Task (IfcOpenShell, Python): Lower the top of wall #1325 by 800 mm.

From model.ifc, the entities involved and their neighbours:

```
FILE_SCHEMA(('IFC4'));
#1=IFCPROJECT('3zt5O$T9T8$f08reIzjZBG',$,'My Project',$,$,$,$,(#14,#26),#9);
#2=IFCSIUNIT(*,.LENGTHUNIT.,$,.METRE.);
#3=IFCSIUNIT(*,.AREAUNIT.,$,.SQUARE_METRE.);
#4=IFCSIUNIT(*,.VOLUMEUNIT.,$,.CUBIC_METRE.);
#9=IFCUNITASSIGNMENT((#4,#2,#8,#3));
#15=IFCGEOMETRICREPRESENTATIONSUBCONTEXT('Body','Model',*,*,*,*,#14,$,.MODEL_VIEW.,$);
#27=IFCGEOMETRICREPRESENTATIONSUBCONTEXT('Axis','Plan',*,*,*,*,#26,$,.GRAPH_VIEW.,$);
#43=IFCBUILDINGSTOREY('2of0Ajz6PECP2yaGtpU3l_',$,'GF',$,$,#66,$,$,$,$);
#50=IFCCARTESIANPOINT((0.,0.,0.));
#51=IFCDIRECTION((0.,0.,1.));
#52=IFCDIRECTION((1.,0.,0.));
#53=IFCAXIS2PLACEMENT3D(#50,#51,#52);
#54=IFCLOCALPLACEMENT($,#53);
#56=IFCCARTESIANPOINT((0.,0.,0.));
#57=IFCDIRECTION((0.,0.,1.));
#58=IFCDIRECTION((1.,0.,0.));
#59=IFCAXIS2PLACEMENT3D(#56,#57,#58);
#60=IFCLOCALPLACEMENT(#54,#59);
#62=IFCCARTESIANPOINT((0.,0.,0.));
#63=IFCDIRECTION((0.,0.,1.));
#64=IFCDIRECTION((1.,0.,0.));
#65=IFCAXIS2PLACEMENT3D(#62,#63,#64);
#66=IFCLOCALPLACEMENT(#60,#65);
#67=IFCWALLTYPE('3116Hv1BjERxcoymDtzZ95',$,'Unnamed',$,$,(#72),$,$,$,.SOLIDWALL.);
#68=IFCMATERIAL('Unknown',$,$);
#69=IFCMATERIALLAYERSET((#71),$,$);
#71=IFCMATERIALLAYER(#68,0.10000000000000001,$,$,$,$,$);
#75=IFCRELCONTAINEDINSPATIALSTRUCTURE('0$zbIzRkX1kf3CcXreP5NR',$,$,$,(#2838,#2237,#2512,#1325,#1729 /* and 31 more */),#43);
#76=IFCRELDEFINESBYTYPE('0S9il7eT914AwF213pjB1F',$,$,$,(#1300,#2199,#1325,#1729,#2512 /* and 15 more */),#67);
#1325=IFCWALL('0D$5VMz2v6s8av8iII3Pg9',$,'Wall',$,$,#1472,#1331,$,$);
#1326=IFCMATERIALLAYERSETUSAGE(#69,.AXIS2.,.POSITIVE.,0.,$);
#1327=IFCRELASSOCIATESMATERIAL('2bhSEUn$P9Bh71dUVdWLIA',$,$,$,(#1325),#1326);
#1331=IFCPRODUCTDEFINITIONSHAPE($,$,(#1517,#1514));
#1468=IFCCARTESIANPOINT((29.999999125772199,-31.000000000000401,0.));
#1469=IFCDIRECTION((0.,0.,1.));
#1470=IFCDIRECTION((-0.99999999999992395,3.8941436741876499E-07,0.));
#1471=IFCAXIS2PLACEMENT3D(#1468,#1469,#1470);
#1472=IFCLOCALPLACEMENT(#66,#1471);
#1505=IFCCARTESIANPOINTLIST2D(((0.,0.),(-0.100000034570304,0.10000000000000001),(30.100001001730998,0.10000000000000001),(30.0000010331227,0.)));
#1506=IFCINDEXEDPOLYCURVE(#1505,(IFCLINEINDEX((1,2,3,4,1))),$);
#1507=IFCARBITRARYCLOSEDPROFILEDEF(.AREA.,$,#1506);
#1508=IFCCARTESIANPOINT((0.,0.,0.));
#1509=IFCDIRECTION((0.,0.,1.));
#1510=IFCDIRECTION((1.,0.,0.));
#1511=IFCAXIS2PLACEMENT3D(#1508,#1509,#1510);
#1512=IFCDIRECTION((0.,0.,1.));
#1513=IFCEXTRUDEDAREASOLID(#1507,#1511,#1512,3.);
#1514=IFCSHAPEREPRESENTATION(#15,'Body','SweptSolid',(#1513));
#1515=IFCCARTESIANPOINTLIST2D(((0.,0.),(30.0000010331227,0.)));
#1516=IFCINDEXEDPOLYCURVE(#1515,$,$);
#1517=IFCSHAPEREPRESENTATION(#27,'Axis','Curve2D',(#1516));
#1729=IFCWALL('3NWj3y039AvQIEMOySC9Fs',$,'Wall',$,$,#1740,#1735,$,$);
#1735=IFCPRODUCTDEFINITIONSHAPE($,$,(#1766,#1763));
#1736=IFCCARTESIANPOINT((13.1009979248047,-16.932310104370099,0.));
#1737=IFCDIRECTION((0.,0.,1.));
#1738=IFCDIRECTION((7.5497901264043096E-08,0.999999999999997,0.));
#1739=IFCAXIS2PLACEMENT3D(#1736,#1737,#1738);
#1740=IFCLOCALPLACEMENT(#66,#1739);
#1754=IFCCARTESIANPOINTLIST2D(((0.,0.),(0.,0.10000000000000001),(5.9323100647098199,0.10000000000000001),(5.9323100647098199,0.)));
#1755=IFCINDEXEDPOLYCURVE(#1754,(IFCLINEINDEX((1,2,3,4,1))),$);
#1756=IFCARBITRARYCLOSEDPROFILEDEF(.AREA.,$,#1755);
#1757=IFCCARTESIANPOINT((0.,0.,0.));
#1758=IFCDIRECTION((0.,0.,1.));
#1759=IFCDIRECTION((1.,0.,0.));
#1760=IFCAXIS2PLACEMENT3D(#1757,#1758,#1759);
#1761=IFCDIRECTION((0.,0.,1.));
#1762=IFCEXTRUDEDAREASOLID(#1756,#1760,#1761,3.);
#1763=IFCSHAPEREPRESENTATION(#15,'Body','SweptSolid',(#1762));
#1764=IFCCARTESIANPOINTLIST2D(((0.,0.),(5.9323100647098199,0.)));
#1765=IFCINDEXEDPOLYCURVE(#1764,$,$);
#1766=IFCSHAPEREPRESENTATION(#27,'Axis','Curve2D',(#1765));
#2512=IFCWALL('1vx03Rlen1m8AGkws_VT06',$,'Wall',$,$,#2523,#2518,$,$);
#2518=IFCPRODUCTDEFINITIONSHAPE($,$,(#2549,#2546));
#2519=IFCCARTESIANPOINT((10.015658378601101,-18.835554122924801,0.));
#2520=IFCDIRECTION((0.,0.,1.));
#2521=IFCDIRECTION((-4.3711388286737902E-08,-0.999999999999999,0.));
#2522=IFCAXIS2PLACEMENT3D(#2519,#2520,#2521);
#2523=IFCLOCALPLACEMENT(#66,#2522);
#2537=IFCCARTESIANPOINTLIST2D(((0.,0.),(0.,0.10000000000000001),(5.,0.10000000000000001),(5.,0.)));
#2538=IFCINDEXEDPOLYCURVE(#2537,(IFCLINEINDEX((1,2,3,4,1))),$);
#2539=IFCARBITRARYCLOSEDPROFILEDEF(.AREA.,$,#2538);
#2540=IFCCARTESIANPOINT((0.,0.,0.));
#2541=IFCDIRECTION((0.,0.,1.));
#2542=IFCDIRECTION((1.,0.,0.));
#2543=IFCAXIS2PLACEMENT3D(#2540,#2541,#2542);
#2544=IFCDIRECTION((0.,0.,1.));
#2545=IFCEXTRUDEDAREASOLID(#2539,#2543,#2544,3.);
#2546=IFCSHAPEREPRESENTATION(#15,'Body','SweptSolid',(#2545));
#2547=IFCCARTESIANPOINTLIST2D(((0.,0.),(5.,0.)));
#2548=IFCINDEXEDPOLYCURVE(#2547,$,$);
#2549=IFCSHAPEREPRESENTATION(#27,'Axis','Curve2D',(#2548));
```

```python
import ifcopenshell
import ifcopenshell.geom
import ifcopenshell.util.representation
import ifcopenshell.util.shape
import ifcopenshell.util.unit

model = ifcopenshell.open("model.ifc")
unit_scale = ifcopenshell.util.unit.calculate_unit_scale(model)
settings = ifcopenshell.geom.settings()


def volume(element):
    """Net volume in cubic metres, openings subtracted."""
    shape = ifcopenshell.geom.create_shape(settings, element)
    return ifcopenshell.util.shape.get_volume(shape.geometry)


wall = model.by_guid("0D$5VMz2v6s8av8iII3Pg9")
before = volume(wall)

body = ifcopenshell.util.representation.get_representation(wall, "Model", "Body")
solid = body.Items[0]
old_height = solid.Depth
solid.Depth -= 0.8 / unit_scale
after = volume(wall)

print(f"height {old_height:g} -> {solid.Depth:g}, volume {before:.3f} -> {after:.3f} m3")

model.write("model_v2.ifc")
```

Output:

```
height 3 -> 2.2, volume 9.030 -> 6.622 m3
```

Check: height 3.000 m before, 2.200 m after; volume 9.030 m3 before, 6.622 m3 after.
